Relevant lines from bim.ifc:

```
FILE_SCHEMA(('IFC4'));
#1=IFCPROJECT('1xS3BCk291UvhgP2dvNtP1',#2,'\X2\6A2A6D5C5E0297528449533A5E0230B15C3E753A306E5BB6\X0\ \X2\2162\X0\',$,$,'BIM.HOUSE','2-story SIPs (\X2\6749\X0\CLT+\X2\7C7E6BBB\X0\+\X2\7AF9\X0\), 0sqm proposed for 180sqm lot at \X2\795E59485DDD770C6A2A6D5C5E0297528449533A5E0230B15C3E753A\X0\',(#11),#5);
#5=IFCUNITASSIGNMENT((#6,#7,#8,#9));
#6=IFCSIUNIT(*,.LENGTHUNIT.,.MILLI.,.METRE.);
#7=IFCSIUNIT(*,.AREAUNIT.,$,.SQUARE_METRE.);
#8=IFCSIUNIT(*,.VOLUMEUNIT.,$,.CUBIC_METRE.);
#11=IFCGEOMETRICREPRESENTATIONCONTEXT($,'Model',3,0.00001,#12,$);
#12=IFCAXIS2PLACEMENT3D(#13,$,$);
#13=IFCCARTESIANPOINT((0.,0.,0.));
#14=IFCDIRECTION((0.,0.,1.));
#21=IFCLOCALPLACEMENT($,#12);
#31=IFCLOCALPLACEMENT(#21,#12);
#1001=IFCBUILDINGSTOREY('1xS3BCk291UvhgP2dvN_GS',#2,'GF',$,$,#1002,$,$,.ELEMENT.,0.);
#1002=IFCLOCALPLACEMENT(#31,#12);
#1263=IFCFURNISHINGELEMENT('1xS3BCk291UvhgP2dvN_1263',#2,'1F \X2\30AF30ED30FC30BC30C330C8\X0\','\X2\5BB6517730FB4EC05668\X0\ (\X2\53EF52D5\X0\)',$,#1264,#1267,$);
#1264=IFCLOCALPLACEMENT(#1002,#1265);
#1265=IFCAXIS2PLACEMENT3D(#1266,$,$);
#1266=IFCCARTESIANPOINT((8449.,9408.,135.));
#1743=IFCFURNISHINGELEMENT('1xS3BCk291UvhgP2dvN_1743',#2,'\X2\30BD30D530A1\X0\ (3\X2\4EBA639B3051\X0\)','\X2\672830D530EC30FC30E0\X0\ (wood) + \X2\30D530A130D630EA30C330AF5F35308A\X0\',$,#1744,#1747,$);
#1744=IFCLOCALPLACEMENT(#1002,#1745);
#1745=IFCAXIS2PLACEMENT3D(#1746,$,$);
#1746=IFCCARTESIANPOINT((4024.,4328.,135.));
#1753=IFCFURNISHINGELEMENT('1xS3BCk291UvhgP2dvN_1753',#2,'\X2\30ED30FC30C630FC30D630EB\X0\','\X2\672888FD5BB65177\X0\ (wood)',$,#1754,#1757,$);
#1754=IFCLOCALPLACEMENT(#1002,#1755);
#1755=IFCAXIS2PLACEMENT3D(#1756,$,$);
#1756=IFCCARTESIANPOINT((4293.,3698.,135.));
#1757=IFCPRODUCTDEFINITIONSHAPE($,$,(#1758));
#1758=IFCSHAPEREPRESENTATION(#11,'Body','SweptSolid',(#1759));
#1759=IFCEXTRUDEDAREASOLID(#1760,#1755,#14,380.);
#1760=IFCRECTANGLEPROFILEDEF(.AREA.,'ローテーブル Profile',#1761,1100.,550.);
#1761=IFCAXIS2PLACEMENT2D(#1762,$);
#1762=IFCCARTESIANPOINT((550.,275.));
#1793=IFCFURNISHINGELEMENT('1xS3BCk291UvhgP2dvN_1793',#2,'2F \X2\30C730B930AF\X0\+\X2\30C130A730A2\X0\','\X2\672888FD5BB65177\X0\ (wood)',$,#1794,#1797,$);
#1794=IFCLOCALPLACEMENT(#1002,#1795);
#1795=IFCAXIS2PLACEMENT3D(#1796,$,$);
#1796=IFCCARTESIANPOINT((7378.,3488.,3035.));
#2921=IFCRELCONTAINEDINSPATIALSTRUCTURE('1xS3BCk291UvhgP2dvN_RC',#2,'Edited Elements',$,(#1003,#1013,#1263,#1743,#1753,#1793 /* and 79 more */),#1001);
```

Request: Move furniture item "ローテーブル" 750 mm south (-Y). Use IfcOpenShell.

```python
import ifcopenshell
import ifcopenshell.api.geometry
import ifcopenshell.util.placement
import ifcopenshell.util.unit

model = ifcopenshell.open("bim.ifc")
unit_scale = ifcopenshell.util.unit.calculate_unit_scale(model)

item = model.by_guid("1xS3BCk291UvhgP2dvN_1753")
matrix = ifcopenshell.util.placement.get_local_placement(item.ObjectPlacement)
matrix[1, 3] -= 0.75 / unit_scale
ifcopenshell.api.geometry.edit_object_placement(model, product=item, matrix=matrix, is_si=False)

print(ifcopenshell.util.placement.get_local_placement(item.ObjectPlacement).round(3) + 0.0)

model.write("bim_edited.ifc")
```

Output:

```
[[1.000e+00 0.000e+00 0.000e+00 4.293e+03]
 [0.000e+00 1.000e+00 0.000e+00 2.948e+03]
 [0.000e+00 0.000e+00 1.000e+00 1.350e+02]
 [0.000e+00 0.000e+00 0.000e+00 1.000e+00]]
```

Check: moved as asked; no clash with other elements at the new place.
